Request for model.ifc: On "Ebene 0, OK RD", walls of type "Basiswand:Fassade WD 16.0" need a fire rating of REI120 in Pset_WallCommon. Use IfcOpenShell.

First a look at what the model holds.

```python
import ifcopenshell
import ifcopenshell.util.element

model = ifcopenshell.open("model.ifc")
print(model.schema)
storey = next(s for s in model.by_type("IfcBuildingStorey") if s.Name == "Ebene 0, OK RD")
walls = [e for e in ifcopenshell.util.element.get_decomposition(storey) if e.is_a("IfcWall")]
seen = {}
for e in walls:
    element_type = ifcopenshell.util.element.get_type(e)
    key = (element_type.Name if element_type != e and element_type else None, ifcopenshell.util.element.get_pset(e, "Pset_WallCommon", "FireRating"))
    seen[key] = seen.get(key, 0) + 1
for (name, value), count in sorted(seen.items(), key=str):
    print(count, "x", name, "|", value)
```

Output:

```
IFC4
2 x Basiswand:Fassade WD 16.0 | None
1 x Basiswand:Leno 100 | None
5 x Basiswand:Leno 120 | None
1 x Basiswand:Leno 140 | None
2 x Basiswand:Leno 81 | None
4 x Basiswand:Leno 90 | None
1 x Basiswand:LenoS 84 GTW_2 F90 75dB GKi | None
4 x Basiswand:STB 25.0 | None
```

```python
import ifcopenshell
import ifcopenshell.api.pset
import ifcopenshell.util.element

model = ifcopenshell.open("model.ifc")

storey = next(s for s in model.by_type("IfcBuildingStorey") if s.Name == "Ebene 0, OK RD")
walls = [e for e in ifcopenshell.util.element.get_decomposition(storey) if e.is_a("IfcWall")]

count = 0
for e in walls:
    element_type = ifcopenshell.util.element.get_type(e)
    if element_type in (None, e) or element_type.Name != "Basiswand:Fassade WD 16.0":
        continue
    # add_pset returns the element's existing set when there is one.
    pset = ifcopenshell.api.pset.add_pset(model, product=e, name="Pset_WallCommon")
    ifcopenshell.api.pset.edit_pset(model, pset=pset, properties={"FireRating": "REI120"})
    count += 1

print(count, "walls updated")

model.write("model_v2.ifc")
```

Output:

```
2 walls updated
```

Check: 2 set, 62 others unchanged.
